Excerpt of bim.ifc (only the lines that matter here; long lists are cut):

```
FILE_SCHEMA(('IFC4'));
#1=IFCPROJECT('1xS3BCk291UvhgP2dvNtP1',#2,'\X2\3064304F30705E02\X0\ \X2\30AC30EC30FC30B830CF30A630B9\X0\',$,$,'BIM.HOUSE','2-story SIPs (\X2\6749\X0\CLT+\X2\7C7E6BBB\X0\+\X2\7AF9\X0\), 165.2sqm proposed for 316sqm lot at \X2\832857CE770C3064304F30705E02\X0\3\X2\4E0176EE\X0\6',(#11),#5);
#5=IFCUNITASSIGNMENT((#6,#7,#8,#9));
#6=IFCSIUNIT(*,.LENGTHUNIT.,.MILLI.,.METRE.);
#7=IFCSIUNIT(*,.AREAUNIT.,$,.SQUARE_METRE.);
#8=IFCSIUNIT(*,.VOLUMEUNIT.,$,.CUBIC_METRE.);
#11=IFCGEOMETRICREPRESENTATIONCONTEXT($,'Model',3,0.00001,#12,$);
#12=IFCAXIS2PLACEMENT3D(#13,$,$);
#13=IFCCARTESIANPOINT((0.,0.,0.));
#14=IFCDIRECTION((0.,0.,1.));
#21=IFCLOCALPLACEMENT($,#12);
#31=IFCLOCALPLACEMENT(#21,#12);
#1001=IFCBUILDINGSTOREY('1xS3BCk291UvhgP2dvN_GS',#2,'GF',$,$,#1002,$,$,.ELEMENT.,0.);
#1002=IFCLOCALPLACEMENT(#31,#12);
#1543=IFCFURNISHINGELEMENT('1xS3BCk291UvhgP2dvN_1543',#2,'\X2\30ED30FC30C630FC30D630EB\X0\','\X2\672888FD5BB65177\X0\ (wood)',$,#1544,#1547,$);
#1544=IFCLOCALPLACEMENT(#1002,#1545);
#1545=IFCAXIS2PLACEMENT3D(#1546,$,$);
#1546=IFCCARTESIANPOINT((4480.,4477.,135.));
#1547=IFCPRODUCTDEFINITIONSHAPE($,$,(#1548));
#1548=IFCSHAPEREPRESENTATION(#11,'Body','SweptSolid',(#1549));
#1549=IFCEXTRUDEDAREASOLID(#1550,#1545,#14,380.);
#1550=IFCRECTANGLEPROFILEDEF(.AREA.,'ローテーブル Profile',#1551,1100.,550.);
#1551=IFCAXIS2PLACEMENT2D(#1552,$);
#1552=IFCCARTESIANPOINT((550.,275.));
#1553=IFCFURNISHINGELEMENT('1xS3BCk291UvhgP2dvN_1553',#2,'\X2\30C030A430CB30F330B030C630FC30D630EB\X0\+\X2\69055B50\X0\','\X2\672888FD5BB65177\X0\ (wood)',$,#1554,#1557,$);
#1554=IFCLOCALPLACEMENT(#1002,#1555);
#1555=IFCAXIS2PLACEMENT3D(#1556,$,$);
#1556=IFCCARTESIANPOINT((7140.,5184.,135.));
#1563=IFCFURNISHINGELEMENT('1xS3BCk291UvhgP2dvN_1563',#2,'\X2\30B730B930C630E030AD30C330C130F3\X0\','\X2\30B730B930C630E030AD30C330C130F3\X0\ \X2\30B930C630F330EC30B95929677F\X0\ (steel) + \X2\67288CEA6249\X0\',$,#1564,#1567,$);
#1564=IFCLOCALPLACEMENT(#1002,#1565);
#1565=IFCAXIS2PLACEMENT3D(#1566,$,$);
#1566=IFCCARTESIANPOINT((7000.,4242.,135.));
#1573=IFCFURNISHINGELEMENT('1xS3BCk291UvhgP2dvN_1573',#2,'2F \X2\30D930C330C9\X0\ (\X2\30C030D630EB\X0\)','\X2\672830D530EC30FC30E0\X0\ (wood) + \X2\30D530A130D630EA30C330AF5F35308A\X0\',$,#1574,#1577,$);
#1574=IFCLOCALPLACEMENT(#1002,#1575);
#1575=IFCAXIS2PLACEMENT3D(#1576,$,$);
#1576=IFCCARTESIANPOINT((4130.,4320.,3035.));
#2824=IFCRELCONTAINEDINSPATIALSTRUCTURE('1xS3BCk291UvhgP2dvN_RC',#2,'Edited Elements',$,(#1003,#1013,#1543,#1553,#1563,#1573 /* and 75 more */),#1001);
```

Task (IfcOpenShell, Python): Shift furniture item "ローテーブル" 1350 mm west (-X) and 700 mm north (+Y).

```python
import ifcopenshell
import ifcopenshell.api.geometry
import ifcopenshell.util.placement
import ifcopenshell.util.unit

model = ifcopenshell.open("bim.ifc")
unit_scale = ifcopenshell.util.unit.calculate_unit_scale(model)

item = model.by_guid("1xS3BCk291UvhgP2dvN_1543")
matrix = ifcopenshell.util.placement.get_local_placement(item.ObjectPlacement)
matrix[0, 3] -= 1.35 / unit_scale
matrix[1, 3] += 0.7 / unit_scale
ifcopenshell.api.geometry.edit_object_placement(model, product=item, matrix=matrix, is_si=False)

print(ifcopenshell.util.placement.get_local_placement(item.ObjectPlacement).round(3) + 0.0)

model.write("bim_updated.ifc")
```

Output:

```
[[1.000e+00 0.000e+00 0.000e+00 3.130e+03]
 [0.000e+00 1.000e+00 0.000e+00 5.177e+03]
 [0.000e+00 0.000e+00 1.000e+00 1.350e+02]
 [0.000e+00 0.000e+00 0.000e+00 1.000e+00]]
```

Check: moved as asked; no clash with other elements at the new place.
